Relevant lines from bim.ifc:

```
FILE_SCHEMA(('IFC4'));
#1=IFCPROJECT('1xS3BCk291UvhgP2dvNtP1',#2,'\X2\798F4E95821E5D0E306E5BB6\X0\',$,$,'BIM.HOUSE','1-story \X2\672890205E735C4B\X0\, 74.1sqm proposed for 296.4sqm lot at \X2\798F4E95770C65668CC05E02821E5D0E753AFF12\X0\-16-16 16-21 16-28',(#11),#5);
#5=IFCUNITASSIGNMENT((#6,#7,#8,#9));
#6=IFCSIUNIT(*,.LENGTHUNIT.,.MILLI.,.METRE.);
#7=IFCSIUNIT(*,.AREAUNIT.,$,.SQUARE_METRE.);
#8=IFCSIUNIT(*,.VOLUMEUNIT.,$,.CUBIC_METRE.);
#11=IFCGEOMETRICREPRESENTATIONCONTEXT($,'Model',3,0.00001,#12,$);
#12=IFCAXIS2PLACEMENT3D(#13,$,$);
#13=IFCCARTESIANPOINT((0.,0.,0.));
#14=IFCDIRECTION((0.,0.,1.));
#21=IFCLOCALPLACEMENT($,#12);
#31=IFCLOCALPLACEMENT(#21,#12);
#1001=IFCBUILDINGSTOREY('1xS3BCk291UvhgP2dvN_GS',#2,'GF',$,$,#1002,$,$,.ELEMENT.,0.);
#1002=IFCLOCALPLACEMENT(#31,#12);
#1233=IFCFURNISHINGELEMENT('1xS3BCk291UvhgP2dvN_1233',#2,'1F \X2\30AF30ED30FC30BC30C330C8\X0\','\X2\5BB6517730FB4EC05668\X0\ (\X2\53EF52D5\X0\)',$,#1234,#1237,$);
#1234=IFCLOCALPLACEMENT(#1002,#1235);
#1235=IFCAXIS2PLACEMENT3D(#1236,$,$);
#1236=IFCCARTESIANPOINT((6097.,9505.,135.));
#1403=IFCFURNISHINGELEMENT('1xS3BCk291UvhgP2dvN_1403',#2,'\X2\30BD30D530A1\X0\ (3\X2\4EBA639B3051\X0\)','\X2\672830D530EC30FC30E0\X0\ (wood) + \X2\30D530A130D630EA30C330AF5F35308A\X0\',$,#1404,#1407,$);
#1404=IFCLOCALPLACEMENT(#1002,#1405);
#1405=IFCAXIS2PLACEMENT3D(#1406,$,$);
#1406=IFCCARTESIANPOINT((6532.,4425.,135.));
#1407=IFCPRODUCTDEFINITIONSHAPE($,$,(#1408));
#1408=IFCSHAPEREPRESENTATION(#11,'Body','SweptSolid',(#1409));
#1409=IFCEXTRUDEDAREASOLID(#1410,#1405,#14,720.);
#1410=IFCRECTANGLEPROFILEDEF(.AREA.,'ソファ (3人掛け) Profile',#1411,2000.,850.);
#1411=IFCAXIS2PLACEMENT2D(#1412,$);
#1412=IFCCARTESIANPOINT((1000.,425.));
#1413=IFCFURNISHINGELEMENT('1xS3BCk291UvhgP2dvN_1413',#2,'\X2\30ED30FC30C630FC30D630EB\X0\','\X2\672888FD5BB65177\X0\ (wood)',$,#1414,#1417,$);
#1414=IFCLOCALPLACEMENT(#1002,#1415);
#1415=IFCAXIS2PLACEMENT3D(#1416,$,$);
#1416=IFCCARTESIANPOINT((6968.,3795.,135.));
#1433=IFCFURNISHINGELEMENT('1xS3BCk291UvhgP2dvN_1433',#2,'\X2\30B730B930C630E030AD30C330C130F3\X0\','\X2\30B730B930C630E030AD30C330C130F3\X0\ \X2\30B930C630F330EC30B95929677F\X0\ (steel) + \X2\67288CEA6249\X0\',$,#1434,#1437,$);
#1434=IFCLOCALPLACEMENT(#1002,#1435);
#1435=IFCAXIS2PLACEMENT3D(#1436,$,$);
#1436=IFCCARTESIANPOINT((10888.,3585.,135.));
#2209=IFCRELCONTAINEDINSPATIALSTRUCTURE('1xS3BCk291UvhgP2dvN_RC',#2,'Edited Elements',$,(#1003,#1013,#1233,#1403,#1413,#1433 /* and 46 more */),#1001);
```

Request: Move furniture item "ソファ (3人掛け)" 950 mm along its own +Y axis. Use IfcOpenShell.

```python
import ifcopenshell
import ifcopenshell.api.geometry
import ifcopenshell.util.placement
import ifcopenshell.util.unit

model = ifcopenshell.open("bim.ifc")
unit_scale = ifcopenshell.util.unit.calculate_unit_scale(model)

item = model.by_id(1403)
matrix = ifcopenshell.util.placement.get_local_placement(item.ObjectPlacement)
matrix[:3, 3] += matrix[:3, 1] * 0.95 / unit_scale
ifcopenshell.api.geometry.edit_object_placement(model, product=item, matrix=matrix, is_si=False)

print(ifcopenshell.util.placement.get_local_placement(item.ObjectPlacement).round(3) + 0.0)

model.write("bim-out.ifc")
```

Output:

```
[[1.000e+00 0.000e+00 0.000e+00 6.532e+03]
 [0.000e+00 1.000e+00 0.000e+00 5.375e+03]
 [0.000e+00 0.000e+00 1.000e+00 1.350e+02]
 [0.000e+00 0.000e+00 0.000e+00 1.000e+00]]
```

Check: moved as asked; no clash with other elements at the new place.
